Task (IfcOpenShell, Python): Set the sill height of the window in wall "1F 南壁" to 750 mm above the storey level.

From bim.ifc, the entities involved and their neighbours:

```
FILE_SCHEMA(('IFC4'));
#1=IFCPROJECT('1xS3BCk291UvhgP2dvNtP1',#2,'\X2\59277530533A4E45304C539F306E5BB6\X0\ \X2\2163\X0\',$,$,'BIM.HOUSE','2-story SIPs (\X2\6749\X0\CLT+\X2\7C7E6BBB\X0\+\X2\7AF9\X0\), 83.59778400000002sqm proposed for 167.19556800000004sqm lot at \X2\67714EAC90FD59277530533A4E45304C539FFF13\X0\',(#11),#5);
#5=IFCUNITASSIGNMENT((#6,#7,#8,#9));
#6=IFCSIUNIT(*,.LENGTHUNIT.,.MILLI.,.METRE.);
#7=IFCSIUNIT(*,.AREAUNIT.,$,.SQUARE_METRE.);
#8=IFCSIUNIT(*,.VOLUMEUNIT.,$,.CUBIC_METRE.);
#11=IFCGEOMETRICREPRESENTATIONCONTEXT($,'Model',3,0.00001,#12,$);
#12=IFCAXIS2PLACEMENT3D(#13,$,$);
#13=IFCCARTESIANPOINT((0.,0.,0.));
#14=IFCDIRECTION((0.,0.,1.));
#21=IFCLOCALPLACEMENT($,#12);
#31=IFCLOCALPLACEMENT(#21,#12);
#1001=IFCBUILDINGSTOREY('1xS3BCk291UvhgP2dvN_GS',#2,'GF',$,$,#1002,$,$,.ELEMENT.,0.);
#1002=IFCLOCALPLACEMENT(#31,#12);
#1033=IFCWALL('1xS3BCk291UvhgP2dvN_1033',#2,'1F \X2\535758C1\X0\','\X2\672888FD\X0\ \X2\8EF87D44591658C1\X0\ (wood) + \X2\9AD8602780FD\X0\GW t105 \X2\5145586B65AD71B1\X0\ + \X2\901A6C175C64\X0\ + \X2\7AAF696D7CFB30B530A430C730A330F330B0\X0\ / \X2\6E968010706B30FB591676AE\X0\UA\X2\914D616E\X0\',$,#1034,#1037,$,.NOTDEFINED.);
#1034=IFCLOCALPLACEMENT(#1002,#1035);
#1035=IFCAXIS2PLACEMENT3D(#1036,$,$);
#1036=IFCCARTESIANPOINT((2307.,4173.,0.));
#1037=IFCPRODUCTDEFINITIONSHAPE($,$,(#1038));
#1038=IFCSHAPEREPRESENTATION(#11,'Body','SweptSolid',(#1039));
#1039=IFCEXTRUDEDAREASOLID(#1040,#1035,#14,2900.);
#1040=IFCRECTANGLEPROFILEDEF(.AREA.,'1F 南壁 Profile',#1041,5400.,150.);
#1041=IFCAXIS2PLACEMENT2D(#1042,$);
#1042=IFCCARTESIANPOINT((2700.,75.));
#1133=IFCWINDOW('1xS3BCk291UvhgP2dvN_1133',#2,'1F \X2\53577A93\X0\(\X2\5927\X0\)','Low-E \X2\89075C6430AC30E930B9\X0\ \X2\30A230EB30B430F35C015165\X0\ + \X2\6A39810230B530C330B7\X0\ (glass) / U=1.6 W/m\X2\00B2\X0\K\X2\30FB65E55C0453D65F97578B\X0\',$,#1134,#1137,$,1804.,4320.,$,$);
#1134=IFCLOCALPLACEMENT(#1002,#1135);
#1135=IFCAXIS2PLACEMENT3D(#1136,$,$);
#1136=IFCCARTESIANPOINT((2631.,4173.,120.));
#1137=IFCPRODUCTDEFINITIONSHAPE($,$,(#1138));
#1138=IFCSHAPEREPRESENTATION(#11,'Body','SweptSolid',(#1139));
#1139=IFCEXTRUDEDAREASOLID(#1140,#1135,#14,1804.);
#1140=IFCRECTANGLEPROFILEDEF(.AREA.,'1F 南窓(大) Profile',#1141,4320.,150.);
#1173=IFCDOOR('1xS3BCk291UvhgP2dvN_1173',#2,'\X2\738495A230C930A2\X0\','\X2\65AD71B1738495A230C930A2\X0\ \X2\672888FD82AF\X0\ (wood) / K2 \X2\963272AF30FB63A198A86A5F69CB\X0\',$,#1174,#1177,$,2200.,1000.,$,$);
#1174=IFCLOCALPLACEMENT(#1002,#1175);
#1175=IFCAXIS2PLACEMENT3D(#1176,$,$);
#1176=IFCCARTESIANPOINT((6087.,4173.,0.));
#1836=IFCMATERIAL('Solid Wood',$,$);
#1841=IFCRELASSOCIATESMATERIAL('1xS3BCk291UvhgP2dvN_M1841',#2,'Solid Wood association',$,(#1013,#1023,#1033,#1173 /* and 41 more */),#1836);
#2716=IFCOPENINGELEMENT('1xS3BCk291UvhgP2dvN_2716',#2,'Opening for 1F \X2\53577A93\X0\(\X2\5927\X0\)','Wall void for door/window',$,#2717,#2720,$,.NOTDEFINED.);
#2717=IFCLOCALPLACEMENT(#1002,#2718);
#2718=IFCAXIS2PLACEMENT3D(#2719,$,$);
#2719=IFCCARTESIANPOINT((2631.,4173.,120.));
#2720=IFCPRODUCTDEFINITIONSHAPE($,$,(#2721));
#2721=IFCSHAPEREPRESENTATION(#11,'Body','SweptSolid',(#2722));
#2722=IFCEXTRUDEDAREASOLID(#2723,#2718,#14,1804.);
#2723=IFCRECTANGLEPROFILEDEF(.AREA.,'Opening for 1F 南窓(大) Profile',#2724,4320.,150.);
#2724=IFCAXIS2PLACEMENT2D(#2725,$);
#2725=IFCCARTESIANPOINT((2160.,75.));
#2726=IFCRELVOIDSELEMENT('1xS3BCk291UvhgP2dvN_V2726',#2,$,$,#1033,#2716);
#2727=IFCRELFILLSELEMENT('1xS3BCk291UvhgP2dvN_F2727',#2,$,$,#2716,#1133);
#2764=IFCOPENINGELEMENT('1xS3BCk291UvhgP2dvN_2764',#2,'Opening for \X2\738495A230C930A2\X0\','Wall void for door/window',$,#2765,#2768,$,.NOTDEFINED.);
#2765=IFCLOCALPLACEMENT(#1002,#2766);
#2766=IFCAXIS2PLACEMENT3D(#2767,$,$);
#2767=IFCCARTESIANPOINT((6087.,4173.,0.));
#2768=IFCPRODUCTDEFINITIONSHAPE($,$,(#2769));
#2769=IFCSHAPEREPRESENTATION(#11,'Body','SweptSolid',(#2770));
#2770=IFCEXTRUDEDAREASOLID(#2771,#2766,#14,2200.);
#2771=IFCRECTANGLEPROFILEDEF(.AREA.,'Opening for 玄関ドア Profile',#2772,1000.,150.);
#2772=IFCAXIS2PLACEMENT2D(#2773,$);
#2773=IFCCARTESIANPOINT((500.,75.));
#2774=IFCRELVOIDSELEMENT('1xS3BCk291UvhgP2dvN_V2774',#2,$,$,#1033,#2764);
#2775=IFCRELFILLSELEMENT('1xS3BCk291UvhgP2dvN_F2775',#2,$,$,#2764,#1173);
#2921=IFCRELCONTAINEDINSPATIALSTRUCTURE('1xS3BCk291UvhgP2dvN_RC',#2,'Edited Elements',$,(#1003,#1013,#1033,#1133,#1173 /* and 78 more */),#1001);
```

```python
import numpy as np
import ifcopenshell
import ifcopenshell.api.geometry
import ifcopenshell.geom
import ifcopenshell.util.element
import ifcopenshell.util.placement
import ifcopenshell.util.shape
import ifcopenshell.util.unit

model = ifcopenshell.open("bim.ifc")
unit_scale = ifcopenshell.util.unit.calculate_unit_scale(model)

window = model.by_guid("1xS3BCk291UvhgP2dvN_1133")
opening = window.FillsVoids[0].RelatingOpeningElement
storey = ifcopenshell.util.element.get_container(window, ifc_class="IfcBuildingStorey")
level = ifcopenshell.util.placement.get_local_placement(storey.ObjectPlacement)[2, 3]

# The opening's origin need not be at the sill, so measure its lowest point.
shape = ifcopenshell.geom.create_shape(ifcopenshell.geom.settings(), opening)
bottom = ifcopenshell.util.shape.get_shape_bottom_elevation(shape, shape.geometry) / unit_scale
dz = level + 0.75 / unit_scale - bottom

shift = np.array([0.0, 0.0, dz])
# The window is not placed relative to its opening, so move both.
for product in (opening, window):
    matrix = ifcopenshell.util.placement.get_local_placement(product.ObjectPlacement)
    matrix[:3, 3] += shift
    ifcopenshell.api.geometry.edit_object_placement(model, product=product, matrix=matrix, is_si=False)

print(f"moved by {dz * unit_scale:+.3f} m")

model.write("bim_rev.ifc")
```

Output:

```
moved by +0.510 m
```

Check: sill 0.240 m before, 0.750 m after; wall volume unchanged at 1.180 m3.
